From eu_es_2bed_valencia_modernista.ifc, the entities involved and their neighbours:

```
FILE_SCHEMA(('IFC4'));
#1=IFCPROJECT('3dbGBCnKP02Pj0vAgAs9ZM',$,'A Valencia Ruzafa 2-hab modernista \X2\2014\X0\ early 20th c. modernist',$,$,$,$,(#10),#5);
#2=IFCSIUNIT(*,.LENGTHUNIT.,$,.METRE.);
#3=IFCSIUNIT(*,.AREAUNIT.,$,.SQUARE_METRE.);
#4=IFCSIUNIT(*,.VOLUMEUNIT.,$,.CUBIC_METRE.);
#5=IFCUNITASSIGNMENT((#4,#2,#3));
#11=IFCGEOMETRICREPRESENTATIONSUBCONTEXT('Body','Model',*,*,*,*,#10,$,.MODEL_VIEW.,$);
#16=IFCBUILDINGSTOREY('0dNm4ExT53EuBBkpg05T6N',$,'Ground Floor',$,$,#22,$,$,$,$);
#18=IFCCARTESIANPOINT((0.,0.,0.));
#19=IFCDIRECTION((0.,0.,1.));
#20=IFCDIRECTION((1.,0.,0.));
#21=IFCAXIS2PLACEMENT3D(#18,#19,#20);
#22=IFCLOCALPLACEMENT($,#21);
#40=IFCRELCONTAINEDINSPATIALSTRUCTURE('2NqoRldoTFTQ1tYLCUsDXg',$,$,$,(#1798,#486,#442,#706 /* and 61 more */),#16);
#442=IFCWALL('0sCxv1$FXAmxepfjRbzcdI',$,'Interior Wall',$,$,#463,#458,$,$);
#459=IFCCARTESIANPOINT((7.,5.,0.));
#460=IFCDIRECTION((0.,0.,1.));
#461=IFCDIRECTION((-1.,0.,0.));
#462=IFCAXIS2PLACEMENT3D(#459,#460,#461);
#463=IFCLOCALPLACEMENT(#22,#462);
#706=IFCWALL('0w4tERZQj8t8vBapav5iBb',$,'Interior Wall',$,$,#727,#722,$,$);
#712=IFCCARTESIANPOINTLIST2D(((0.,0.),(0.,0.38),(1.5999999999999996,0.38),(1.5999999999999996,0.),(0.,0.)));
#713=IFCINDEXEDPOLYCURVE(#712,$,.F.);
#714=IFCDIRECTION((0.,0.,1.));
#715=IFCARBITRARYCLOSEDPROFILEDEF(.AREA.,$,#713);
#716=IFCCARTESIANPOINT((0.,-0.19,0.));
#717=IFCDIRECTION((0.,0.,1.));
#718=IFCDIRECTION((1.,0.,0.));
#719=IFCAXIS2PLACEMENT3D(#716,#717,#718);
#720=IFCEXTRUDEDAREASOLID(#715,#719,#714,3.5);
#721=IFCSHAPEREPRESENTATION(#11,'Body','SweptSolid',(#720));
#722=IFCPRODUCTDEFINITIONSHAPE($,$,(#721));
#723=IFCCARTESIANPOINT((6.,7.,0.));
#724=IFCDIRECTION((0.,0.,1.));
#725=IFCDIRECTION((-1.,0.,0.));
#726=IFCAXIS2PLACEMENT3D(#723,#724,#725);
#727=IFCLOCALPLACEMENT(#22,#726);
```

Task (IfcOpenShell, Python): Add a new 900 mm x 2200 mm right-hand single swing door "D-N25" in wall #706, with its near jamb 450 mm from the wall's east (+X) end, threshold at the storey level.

```python
import numpy as np
import ifcopenshell
import ifcopenshell.api.feature
import ifcopenshell.api.geometry
import ifcopenshell.api.root
import ifcopenshell.api.spatial
import ifcopenshell.geom
import ifcopenshell.util.element
import ifcopenshell.util.placement
import ifcopenshell.util.representation
import ifcopenshell.util.shape
import ifcopenshell.util.unit

model = ifcopenshell.open("eu_es_2bed_valencia_modernista.ifc")
unit_scale = ifcopenshell.util.unit.calculate_unit_scale(model)
settings = ifcopenshell.geom.settings()


def volume(element):
    """Net volume in cubic metres, openings subtracted."""
    shape = ifcopenshell.geom.create_shape(settings, element)
    return ifcopenshell.util.shape.get_volume(shape.geometry)


wall = model.by_guid("0w4tERZQj8t8vBapav5iBb")
storey = ifcopenshell.util.element.get_container(wall, ifc_class="IfcBuildingStorey")
context = ifcopenshell.util.representation.get_context(model, "Model", "Body", "MODEL_VIEW")
before = volume(wall)

width, height, from_end, sill = 0.9, 2.2, 0.45, 0.0  # metres

# The wall runs along its own X axis, and the end named is its -X end.
wall_shape = ifcopenshell.geom.create_shape(settings, wall)
x, y, z = ifcopenshell.util.shape.get_vertices(wall_shape.geometry).T
start = x.min() + from_end
face, thickness = float(y.min()), float(y.max() - y.min())
wall_matrix = ifcopenshell.util.placement.get_local_placement(wall.ObjectPlacement)
level = ifcopenshell.util.placement.get_local_placement(storey.ObjectPlacement)[2, 3]


def in_wall(x, y):
    """Placement at x, y metres in the wall's axes, at sill height."""
    matrix = wall_matrix.copy()
    matrix[:, 3] = wall_matrix @ np.array([x / unit_scale, y / unit_scale, 0.0, 1.0])
    matrix[2, 3] = level + sill / unit_scale
    return matrix


# Opening: a box that overshoots both wall faces by 50 mm.
opening = ifcopenshell.api.root.create_entity(model, ifc_class="IfcOpeningElement", predefined_type="OPENING")
box = ifcopenshell.api.geometry.add_wall_representation(
    model, context=context, length=width, height=height, thickness=thickness + 0.1
)
ifcopenshell.api.geometry.assign_representation(model, product=opening, representation=box)
ifcopenshell.api.geometry.edit_object_placement(model, product=opening, matrix=in_wall(start, face - 0.05), is_si=False)
ifcopenshell.api.feature.add_feature(model, feature=opening, element=wall)

door = ifcopenshell.api.root.create_entity(model, ifc_class="IfcDoor", name="D-N25", predefined_type="DOOR")
door.OverallWidth, door.OverallHeight = width / unit_scale, height / unit_scale
door.OperationType = "SINGLE_SWING_RIGHT"
body = ifcopenshell.api.geometry.add_door_representation(
    model,
    context=context,
    overall_width=door.OverallWidth,
    overall_height=door.OverallHeight,
    operation_type="SINGLE_SWING_RIGHT",
    lining_properties={"LiningDepth": thickness / unit_scale, "ThresholdDepth": thickness / unit_scale},
)
ifcopenshell.api.geometry.assign_representation(model, product=door, representation=body)
ifcopenshell.api.spatial.assign_container(model, products=[door], relating_structure=storey)
ifcopenshell.api.feature.add_filling(model, opening=opening, element=door)

# The lining spans the wall, so the door starts at the wall face.
ifcopenshell.api.geometry.edit_object_placement(model, product=door, matrix=in_wall(start, face), is_si=False)

after = volume(wall)

print(f"wall volume {before:.3f} -> {after:.3f} m3")

model.write("eu_es_2bed_valencia_modernista_v2.ifc")
```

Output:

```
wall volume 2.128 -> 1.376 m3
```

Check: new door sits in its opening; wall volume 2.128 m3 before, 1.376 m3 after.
